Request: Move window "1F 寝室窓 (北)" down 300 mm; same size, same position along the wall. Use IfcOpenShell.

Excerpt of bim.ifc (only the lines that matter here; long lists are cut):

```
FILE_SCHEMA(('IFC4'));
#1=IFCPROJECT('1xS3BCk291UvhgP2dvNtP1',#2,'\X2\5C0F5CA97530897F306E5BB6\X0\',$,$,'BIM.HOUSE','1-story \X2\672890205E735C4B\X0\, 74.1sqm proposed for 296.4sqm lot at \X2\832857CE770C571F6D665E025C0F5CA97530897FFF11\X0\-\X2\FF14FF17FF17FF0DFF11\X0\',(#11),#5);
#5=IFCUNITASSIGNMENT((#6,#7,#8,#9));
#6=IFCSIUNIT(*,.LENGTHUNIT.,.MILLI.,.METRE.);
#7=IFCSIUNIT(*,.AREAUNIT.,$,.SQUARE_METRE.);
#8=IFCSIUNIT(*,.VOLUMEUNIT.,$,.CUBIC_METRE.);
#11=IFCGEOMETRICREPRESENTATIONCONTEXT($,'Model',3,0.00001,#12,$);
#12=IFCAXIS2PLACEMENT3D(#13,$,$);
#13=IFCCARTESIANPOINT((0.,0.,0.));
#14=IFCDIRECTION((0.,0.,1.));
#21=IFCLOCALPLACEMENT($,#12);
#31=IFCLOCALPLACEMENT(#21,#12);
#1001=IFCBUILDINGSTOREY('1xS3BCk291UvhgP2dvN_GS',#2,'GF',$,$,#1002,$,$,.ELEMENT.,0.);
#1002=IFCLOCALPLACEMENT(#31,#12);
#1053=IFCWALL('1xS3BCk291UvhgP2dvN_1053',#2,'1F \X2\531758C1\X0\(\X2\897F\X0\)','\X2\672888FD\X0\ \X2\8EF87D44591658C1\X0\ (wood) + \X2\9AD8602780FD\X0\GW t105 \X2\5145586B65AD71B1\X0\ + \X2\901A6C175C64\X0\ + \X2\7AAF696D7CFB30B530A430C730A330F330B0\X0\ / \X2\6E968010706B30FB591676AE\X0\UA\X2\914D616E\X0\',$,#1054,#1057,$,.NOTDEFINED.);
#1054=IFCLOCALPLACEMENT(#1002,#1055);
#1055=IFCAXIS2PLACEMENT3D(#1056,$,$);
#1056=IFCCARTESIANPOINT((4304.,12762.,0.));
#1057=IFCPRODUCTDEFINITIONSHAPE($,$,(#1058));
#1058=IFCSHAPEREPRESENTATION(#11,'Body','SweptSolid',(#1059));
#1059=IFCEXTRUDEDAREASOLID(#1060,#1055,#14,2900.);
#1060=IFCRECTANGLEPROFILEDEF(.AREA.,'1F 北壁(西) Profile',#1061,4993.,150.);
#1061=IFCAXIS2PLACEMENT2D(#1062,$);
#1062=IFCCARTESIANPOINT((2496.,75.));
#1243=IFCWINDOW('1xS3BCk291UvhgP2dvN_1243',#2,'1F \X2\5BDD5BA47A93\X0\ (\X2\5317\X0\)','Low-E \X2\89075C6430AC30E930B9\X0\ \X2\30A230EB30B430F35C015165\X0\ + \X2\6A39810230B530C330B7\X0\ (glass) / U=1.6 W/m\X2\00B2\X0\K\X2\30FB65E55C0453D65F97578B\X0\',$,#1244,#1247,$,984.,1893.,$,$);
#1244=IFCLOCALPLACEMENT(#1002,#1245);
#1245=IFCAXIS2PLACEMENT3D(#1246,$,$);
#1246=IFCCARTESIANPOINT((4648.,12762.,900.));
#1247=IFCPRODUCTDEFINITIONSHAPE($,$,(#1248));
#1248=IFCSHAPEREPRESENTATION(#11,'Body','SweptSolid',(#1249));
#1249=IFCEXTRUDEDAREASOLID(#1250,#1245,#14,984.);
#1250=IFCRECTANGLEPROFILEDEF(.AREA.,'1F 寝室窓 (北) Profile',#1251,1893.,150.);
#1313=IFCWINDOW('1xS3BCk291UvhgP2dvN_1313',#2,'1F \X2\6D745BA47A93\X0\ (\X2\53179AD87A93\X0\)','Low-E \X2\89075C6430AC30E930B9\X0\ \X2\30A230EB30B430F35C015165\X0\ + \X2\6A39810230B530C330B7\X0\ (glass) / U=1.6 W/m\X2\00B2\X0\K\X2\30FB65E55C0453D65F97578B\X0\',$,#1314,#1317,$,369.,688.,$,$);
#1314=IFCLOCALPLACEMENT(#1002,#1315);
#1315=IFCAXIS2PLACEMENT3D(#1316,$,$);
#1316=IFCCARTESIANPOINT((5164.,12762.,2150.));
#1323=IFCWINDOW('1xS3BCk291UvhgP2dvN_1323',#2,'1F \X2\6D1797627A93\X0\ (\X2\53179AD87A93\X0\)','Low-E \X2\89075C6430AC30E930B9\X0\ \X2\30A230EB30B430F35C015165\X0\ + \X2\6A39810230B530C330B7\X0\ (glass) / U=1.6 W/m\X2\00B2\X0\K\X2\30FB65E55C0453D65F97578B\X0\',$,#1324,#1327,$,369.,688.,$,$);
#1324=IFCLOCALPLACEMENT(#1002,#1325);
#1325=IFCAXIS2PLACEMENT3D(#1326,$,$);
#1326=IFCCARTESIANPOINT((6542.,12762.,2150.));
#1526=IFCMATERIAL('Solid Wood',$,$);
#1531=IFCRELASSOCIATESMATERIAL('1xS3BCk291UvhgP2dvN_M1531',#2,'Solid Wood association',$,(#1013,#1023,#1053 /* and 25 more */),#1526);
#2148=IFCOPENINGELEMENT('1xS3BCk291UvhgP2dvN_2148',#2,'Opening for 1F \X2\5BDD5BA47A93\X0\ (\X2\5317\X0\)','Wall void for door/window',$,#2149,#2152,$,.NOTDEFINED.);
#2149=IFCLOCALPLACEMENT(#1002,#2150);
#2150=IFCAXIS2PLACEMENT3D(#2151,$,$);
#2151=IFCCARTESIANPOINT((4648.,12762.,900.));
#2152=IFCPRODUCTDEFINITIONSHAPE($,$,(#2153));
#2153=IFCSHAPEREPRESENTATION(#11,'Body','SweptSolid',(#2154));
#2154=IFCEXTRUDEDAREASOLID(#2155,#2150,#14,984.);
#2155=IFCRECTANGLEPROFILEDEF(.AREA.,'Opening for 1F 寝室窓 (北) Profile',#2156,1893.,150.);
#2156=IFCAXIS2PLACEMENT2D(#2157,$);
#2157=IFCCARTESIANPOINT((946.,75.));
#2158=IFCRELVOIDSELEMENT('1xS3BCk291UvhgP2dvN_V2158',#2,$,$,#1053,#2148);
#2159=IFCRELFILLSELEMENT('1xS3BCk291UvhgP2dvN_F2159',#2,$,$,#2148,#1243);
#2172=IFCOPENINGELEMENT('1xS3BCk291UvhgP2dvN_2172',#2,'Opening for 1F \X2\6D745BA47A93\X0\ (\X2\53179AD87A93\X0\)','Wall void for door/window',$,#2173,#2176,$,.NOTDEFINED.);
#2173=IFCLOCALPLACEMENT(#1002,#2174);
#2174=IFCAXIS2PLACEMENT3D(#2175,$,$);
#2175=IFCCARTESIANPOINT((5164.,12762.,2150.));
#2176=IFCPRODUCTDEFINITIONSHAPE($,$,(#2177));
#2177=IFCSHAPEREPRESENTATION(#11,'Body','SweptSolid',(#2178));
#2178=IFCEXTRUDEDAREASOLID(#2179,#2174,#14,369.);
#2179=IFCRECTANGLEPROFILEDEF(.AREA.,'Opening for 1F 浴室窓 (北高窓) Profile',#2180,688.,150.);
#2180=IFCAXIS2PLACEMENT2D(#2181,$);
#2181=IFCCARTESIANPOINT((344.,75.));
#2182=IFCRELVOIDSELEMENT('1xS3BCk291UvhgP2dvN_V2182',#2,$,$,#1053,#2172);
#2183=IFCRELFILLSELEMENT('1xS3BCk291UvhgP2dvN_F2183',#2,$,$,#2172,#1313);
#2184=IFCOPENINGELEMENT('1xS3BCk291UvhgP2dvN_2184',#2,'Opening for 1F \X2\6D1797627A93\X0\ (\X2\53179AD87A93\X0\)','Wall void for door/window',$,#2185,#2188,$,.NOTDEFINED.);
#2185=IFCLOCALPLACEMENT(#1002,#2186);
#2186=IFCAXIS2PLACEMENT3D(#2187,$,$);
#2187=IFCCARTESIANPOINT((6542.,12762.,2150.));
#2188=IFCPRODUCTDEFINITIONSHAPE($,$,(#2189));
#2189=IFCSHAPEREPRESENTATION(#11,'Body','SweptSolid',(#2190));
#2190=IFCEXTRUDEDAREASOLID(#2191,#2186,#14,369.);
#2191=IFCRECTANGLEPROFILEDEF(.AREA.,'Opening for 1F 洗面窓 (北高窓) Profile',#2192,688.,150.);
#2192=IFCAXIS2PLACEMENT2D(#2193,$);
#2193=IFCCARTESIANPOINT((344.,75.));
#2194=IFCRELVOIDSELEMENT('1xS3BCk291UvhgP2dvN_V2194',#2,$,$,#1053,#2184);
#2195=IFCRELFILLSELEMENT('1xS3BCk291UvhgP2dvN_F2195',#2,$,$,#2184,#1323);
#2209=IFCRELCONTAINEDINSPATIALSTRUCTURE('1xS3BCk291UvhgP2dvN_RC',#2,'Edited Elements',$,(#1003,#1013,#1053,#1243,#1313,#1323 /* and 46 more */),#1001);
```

```python
import numpy as np
import ifcopenshell
import ifcopenshell.api.geometry
import ifcopenshell.util.placement
import ifcopenshell.util.unit

model = ifcopenshell.open("bim.ifc")
unit_scale = ifcopenshell.util.unit.calculate_unit_scale(model)

window = model.by_id(1243)
opening = window.FillsVoids[0].RelatingOpeningElement
dz = -0.3 / unit_scale

shift = np.array([0.0, 0.0, dz])
# The window is not placed relative to its opening, so move both.
for product in (opening, window):
    matrix = ifcopenshell.util.placement.get_local_placement(product.ObjectPlacement)
    matrix[:3, 3] += shift
    ifcopenshell.api.geometry.edit_object_placement(model, product=product, matrix=matrix, is_si=False)

print(f"moved by {dz * unit_scale:+.3f} m")

model.write("bim_edited.ifc")
```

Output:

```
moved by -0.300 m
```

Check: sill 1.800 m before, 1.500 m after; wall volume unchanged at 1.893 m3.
